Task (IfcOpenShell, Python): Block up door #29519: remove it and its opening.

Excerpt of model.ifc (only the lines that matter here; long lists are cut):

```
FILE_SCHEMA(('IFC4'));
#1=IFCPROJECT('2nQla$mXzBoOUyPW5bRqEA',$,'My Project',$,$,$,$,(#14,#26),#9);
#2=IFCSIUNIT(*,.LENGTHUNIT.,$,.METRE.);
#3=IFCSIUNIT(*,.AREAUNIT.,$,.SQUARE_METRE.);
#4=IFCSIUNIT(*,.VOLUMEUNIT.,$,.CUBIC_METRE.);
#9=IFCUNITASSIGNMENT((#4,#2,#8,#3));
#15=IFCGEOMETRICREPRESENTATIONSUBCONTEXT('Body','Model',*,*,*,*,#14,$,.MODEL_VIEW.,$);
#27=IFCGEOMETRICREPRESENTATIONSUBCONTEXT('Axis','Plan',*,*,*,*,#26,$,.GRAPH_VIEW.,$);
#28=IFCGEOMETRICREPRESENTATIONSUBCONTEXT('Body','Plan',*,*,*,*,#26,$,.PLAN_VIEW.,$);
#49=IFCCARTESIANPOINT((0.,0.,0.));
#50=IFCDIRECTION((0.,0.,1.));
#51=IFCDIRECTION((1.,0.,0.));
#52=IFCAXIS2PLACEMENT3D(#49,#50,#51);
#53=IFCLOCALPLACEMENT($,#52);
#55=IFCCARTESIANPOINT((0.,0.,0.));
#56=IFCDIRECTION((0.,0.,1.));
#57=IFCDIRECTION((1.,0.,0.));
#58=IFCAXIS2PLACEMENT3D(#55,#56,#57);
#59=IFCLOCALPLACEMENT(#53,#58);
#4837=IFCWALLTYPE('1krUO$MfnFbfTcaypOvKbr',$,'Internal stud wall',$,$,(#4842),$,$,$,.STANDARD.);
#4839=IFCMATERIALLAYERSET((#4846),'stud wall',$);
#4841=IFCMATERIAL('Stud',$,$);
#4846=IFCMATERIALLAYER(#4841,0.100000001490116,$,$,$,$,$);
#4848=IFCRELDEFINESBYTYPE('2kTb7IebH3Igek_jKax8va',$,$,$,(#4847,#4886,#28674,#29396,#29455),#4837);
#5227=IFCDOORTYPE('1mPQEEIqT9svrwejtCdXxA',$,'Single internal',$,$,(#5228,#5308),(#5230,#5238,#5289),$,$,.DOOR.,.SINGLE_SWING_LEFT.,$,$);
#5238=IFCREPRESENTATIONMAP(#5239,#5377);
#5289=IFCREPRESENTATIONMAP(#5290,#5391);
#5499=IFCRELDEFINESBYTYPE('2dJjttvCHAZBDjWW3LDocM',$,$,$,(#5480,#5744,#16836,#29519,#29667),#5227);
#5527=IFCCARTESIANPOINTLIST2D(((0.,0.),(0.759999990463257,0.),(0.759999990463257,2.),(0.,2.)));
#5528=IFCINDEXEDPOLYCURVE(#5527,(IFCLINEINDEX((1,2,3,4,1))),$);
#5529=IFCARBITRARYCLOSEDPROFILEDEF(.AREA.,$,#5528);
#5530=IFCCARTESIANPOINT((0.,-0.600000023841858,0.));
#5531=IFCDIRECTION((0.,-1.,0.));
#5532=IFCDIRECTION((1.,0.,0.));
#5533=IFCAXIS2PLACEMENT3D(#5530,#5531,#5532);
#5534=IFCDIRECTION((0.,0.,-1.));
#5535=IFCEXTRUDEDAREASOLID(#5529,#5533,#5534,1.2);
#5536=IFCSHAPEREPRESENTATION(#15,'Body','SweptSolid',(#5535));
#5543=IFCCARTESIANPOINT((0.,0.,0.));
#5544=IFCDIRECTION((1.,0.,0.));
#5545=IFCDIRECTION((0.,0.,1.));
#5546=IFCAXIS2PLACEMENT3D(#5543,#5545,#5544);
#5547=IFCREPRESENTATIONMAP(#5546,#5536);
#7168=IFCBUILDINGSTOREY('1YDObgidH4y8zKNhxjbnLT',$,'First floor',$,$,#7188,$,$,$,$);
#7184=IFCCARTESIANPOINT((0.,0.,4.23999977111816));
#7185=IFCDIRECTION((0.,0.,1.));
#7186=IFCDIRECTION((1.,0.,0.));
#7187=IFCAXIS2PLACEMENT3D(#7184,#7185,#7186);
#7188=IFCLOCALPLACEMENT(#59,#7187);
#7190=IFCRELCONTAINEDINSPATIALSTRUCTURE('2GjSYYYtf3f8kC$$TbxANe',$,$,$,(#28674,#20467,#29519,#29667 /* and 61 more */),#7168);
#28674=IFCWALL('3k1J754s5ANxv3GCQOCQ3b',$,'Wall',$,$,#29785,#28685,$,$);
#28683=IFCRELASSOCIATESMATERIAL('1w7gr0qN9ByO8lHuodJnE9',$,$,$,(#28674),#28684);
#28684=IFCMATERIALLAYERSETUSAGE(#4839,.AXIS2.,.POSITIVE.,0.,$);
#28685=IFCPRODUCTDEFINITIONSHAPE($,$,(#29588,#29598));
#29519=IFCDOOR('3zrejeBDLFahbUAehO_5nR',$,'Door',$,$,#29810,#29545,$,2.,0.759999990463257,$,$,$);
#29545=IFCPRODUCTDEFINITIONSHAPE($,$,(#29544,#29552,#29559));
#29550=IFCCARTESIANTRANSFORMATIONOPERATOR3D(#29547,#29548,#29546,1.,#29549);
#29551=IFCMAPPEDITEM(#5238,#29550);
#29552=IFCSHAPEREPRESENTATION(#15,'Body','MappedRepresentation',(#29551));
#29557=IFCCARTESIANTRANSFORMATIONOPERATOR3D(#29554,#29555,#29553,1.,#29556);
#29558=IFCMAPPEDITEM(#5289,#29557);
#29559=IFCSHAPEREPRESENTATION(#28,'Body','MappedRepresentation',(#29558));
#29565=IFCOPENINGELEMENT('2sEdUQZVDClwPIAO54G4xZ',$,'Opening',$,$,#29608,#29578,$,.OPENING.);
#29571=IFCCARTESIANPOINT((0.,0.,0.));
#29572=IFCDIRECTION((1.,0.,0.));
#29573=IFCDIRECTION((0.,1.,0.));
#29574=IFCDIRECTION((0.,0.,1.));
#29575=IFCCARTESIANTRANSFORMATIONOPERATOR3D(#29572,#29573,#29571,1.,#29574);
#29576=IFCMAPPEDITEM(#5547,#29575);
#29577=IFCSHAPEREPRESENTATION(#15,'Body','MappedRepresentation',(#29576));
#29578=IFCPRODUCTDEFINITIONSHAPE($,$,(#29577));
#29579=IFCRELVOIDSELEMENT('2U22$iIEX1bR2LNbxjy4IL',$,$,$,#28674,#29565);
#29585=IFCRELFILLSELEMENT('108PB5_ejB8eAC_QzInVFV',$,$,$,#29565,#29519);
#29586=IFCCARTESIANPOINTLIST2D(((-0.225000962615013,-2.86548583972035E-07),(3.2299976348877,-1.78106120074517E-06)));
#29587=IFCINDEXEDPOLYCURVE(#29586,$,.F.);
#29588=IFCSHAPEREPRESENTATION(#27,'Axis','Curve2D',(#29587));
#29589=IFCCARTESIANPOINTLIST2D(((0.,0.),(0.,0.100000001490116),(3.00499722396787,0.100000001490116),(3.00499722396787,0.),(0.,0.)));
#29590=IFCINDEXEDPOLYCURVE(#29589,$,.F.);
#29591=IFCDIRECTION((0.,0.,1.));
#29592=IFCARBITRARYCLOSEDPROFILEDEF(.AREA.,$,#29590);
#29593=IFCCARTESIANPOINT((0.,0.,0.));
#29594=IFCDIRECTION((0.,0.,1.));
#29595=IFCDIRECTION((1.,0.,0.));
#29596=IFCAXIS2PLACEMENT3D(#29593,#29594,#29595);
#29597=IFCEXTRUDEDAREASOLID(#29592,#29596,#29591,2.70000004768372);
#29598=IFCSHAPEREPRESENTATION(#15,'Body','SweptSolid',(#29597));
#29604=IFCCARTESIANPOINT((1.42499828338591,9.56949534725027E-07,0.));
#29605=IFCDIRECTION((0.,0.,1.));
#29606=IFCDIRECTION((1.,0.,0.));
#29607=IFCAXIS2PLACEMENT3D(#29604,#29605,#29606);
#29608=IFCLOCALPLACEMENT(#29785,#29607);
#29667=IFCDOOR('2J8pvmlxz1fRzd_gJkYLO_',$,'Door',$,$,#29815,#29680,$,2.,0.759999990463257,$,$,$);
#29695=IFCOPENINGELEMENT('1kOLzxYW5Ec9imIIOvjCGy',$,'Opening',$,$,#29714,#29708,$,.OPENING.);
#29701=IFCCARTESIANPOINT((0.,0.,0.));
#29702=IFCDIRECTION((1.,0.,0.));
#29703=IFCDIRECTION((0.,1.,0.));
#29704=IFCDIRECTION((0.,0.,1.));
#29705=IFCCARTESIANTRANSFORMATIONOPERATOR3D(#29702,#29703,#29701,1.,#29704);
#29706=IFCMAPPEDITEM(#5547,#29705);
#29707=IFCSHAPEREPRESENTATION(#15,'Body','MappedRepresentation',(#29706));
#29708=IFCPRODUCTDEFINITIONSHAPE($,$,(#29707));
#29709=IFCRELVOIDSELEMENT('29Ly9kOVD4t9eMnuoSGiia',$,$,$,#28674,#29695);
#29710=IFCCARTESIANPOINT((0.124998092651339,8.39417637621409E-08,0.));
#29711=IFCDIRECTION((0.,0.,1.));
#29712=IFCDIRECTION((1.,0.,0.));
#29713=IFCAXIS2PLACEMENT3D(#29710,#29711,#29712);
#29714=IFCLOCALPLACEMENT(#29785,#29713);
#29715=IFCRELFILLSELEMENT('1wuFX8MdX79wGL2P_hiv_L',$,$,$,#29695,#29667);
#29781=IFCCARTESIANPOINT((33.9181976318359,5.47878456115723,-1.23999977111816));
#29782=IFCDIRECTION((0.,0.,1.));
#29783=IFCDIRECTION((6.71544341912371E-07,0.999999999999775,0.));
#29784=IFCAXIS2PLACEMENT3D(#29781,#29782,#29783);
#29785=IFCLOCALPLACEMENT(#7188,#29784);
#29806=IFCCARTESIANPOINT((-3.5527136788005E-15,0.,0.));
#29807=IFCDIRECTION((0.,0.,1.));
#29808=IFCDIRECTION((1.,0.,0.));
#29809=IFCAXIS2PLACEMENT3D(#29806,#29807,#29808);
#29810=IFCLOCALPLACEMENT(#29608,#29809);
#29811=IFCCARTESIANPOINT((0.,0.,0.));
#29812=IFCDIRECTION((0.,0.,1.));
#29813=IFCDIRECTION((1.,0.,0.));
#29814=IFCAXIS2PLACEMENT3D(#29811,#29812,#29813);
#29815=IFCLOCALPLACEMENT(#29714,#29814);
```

```python
import ifcopenshell
import ifcopenshell.api.feature
import ifcopenshell.api.root
import ifcopenshell.geom
import ifcopenshell.util.shape

model = ifcopenshell.open("model.ifc")
settings = ifcopenshell.geom.settings()


def volume(element):
    """Net volume in cubic metres, openings subtracted."""
    shape = ifcopenshell.geom.create_shape(settings, element)
    return ifcopenshell.util.shape.get_volume(shape.geometry)


door = model.by_id(29519)
opening = door.FillsVoids[0].RelatingOpeningElement
wall = opening.VoidsElements[0].RelatingBuildingElement
before = volume(wall)

ifcopenshell.api.root.remove_product(model, product=door)
ifcopenshell.api.feature.remove_feature(model, feature=opening)

after = volume(wall)

print(f"wall volume {before:.3f} -> {after:.3f} m3")

model.write("model_edited.ifc")
```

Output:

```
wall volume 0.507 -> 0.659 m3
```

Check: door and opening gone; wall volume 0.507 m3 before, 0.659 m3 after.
